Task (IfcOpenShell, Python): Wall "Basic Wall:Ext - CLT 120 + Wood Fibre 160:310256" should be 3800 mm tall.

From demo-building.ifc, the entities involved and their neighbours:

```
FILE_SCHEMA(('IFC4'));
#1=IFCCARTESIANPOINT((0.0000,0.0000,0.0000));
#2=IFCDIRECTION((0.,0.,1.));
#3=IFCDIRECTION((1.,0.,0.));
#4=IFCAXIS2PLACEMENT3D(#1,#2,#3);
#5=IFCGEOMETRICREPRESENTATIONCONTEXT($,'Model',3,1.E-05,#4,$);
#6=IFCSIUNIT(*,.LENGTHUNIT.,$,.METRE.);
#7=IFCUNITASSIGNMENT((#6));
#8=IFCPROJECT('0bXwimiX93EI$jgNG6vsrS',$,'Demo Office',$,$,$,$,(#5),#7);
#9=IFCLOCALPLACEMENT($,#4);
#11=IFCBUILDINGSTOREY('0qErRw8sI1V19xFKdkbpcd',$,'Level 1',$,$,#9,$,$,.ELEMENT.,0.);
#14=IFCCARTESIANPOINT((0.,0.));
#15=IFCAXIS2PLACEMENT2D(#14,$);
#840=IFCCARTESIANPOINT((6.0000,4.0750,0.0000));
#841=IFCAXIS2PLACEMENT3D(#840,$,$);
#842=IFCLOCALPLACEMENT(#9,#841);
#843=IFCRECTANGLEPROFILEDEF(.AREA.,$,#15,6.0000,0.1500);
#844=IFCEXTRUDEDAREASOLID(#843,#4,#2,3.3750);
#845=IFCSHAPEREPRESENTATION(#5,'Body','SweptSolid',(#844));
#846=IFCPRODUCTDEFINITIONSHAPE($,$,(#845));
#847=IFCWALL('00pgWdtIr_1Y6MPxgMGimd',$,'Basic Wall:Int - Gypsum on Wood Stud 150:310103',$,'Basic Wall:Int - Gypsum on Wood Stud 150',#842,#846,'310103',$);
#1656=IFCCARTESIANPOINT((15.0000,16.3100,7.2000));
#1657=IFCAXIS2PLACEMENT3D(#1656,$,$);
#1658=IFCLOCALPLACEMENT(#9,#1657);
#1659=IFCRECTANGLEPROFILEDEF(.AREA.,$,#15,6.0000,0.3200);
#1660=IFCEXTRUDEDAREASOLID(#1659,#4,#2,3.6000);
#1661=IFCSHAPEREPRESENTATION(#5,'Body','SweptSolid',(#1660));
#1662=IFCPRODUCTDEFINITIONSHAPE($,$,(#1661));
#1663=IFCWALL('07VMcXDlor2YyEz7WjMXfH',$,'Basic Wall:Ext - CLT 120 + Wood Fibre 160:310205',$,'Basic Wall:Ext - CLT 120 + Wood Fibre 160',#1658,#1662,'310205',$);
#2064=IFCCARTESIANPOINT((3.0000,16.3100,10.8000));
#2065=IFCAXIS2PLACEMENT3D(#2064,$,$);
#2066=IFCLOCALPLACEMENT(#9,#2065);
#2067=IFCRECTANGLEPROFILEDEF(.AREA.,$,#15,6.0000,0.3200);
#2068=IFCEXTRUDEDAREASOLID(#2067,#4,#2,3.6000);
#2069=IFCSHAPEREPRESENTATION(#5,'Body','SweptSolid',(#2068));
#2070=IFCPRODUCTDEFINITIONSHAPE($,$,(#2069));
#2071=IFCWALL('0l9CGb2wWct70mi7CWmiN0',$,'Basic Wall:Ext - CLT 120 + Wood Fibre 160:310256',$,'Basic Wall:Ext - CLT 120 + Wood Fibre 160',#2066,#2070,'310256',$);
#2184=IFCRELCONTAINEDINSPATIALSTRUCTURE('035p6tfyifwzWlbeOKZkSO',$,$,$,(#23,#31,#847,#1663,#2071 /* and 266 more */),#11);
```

```python
import ifcopenshell
import ifcopenshell.geom
import ifcopenshell.util.shape
import ifcopenshell.util.unit

model = ifcopenshell.open("demo-building.ifc")
unit_scale = ifcopenshell.util.unit.calculate_unit_scale(model)
settings = ifcopenshell.geom.settings()


def volume(element):
    """Net volume in cubic metres, openings subtracted."""
    shape = ifcopenshell.geom.create_shape(settings, element)
    return ifcopenshell.util.shape.get_volume(shape.geometry)


wall = model.by_id(2071)
before = volume(wall)

body = next(r for r in wall.Representation.Representations if r.RepresentationIdentifier == "Body")
solid = body.Items[0]
old_height = solid.Depth
solid.Depth = 3.8 / unit_scale
after = volume(wall)

print(f"height {old_height:g} -> {solid.Depth:g}, volume {before:.3f} -> {after:.3f} m3")

model.write("demo-building_v2.ifc")
```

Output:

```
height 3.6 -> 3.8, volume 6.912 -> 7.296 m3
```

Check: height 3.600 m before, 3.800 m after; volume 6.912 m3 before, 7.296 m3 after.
